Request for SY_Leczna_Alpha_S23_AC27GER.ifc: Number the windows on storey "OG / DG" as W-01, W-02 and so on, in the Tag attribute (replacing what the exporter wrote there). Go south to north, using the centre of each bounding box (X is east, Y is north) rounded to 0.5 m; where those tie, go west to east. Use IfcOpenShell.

First a look at what the model holds.

```python
import ifcopenshell
import ifcopenshell.util.element
import ifcopenshell.util.placement

model = ifcopenshell.open("SY_Leczna_Alpha_S23_AC27GER.ifc")
print(model.schema)
storey = next(s for s in model.by_type("IfcBuildingStorey") if s.Name == "OG / DG")
windows = [e for e in ifcopenshell.util.element.get_decomposition(storey) if e.is_a("IfcWindow")]
for e in sorted(windows, key=lambda e: e.id()):
    origin = ifcopenshell.util.placement.get_local_placement(e.ObjectPlacement)[:3, 3]
    print(e.id(), e.Tag, e.Name, origin.round(2) + 0.0, sep=" | ")
```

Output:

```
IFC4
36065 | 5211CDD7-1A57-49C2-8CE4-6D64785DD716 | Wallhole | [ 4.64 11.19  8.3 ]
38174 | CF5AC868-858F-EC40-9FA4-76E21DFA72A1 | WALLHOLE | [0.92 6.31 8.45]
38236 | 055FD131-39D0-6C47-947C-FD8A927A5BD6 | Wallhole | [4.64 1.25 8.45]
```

```python
import ifcopenshell
import ifcopenshell.geom
import ifcopenshell.util.element
import ifcopenshell.util.shape

model = ifcopenshell.open("SY_Leczna_Alpha_S23_AC27GER.ifc")
settings = ifcopenshell.geom.settings()
settings.set("use-world-coords", True)


def centre(element):
    shape = ifcopenshell.geom.create_shape(settings, element)
    return ifcopenshell.util.shape.get_bbox_centroid(shape.geometry)


storey = next(s for s in model.by_type("IfcBuildingStorey") if s.Name == "OG / DG")
windows = [e for e in ifcopenshell.util.element.get_decomposition(storey) if e.is_a("IfcWindow")]

# Insertion points can sit at a corner or the storey origin, so sort by the geometry (in metres).
centres = {e: centre(e) for e in windows}
windows.sort(key=lambda e: (round(centres[e][1] / 0.5), centres[e][0]))

for i, e in enumerate(windows, start=1):
    number = f"W-{i:02d}"
    e.Tag = number
    print(e.id(), number)

model.write("SY_Leczna_Alpha_S23_AC27GER_v2.ifc")
```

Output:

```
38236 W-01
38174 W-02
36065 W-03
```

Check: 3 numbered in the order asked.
